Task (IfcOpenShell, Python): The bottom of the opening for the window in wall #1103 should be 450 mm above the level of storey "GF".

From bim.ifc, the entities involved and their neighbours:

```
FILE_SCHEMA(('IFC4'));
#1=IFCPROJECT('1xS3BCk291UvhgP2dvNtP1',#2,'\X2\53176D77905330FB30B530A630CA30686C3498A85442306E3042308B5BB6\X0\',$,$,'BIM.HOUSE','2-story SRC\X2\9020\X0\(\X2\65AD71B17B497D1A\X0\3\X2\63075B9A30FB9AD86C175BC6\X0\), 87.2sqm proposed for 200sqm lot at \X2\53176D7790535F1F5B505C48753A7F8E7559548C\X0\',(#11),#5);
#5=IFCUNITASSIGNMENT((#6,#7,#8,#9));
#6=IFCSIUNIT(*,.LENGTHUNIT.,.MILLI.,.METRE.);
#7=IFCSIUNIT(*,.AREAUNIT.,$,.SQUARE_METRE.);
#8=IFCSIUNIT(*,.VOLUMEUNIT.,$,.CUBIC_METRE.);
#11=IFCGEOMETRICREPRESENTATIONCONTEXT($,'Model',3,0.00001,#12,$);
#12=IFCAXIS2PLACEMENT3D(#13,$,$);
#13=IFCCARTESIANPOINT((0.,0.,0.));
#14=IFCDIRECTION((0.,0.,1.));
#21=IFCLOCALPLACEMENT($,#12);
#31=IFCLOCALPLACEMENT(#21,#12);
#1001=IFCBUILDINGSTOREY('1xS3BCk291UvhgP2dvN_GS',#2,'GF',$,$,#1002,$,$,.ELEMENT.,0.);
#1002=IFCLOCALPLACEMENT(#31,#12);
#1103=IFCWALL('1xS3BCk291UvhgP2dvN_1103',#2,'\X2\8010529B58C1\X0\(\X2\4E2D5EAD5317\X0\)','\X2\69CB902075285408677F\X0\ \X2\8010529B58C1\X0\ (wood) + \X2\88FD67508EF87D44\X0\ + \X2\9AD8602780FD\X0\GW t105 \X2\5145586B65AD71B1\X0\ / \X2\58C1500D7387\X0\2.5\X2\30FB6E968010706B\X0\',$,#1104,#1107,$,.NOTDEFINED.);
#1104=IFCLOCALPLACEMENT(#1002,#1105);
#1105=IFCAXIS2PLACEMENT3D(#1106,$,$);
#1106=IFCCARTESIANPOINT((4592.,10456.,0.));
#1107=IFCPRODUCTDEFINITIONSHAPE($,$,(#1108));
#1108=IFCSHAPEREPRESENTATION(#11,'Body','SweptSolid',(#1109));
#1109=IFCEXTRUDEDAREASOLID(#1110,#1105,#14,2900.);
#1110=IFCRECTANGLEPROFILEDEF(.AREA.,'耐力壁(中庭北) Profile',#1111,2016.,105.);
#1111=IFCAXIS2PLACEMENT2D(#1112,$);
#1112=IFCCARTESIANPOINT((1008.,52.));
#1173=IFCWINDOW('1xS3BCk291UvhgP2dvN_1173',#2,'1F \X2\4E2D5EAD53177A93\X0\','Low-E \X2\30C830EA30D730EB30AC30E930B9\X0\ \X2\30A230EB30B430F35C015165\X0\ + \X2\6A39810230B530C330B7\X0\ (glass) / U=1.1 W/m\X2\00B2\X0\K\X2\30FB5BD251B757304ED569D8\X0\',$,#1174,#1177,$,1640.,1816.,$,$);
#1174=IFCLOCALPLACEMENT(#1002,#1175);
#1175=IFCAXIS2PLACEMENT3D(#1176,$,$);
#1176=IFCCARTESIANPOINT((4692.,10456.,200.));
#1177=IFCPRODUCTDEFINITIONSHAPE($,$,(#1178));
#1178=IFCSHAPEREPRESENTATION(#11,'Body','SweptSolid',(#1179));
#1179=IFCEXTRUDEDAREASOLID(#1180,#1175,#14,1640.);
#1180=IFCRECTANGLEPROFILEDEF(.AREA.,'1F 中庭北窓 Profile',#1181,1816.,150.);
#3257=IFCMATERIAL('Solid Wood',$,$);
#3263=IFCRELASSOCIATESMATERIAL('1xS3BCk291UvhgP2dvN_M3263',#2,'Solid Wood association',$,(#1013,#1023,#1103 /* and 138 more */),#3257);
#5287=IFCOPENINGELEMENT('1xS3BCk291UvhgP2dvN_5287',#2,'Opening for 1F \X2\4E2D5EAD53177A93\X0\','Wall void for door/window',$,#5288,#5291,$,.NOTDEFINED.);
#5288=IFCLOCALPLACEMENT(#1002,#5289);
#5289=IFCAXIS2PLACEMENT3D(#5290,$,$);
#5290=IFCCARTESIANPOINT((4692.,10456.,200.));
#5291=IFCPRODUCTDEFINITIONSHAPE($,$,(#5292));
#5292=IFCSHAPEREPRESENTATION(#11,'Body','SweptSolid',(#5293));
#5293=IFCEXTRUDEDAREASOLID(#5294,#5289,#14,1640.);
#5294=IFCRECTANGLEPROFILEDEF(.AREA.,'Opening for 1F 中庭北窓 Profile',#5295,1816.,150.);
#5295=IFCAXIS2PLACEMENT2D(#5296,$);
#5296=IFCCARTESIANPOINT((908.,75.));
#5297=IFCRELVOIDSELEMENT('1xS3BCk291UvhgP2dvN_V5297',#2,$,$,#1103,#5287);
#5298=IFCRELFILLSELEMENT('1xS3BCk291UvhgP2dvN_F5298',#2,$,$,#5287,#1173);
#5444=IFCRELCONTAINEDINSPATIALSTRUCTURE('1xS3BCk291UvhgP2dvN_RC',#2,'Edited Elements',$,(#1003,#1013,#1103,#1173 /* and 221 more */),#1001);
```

```python
import numpy as np
import ifcopenshell
import ifcopenshell.api.geometry
import ifcopenshell.geom
import ifcopenshell.util.element
import ifcopenshell.util.placement
import ifcopenshell.util.shape
import ifcopenshell.util.unit

model = ifcopenshell.open("bim.ifc")
unit_scale = ifcopenshell.util.unit.calculate_unit_scale(model)

window = model.by_guid("1xS3BCk291UvhgP2dvN_1173")
opening = window.FillsVoids[0].RelatingOpeningElement
storey = ifcopenshell.util.element.get_container(window, ifc_class="IfcBuildingStorey")
level = ifcopenshell.util.placement.get_local_placement(storey.ObjectPlacement)[2, 3]

# The opening's origin need not be at the sill, so measure its lowest point.
shape = ifcopenshell.geom.create_shape(ifcopenshell.geom.settings(), opening)
bottom = ifcopenshell.util.shape.get_shape_bottom_elevation(shape, shape.geometry) / unit_scale
dz = level + 0.45 / unit_scale - bottom

shift = np.array([0.0, 0.0, dz])
# The window is not placed relative to its opening, so move both.
for product in (opening, window):
    matrix = ifcopenshell.util.placement.get_local_placement(product.ObjectPlacement)
    matrix[:3, 3] += shift
    ifcopenshell.api.geometry.edit_object_placement(model, product=product, matrix=matrix, is_si=False)

print(f"moved by {dz * unit_scale:+.3f} m")

model.write("bim-out.ifc")
```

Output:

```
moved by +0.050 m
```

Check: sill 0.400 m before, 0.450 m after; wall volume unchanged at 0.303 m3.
